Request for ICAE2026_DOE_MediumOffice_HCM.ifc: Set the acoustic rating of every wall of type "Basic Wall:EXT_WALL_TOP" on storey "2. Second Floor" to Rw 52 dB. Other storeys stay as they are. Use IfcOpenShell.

First a look at what the model holds.

```python
import ifcopenshell
import ifcopenshell.util.element

model = ifcopenshell.open("ICAE2026_DOE_MediumOffice_HCM.ifc")
print(model.schema)
storey = next(s for s in model.by_type("IfcBuildingStorey") if s.Name == "2. Second Floor")
walls = [e for e in ifcopenshell.util.element.get_decomposition(storey) if e.is_a("IfcWall")]
seen = {}
for e in walls:
    element_type = ifcopenshell.util.element.get_type(e)
    key = (element_type.Name if element_type != e and element_type else None, ifcopenshell.util.element.get_pset(e, "Pset_WallCommon", "AcousticRating"))
    seen[key] = seen.get(key, 0) + 1
for (name, value), count in sorted(seen.items(), key=str):
    print(count, "x", name, "|", value)
```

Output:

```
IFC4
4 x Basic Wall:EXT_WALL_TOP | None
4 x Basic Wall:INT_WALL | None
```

```python
import ifcopenshell
import ifcopenshell.api.pset
import ifcopenshell.util.element

model = ifcopenshell.open("ICAE2026_DOE_MediumOffice_HCM.ifc")

storey = next(s for s in model.by_type("IfcBuildingStorey") if s.Name == "2. Second Floor")
walls = [e for e in ifcopenshell.util.element.get_decomposition(storey) if e.is_a("IfcWall")]

count = 0
for e in walls:
    element_type = ifcopenshell.util.element.get_type(e)
    if element_type in (None, e) or element_type.Name != "Basic Wall:EXT_WALL_TOP":
        continue
    # add_pset returns the element's existing set when there is one.
    pset = ifcopenshell.api.pset.add_pset(model, product=e, name="Pset_WallCommon")
    ifcopenshell.api.pset.edit_pset(model, pset=pset, properties={"AcousticRating": "Rw 52 dB"})
    count += 1

print(count, "walls updated")

model.write("ICAE2026_DOE_MediumOffice_HCM_rev.ifc")
```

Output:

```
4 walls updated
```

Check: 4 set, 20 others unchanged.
